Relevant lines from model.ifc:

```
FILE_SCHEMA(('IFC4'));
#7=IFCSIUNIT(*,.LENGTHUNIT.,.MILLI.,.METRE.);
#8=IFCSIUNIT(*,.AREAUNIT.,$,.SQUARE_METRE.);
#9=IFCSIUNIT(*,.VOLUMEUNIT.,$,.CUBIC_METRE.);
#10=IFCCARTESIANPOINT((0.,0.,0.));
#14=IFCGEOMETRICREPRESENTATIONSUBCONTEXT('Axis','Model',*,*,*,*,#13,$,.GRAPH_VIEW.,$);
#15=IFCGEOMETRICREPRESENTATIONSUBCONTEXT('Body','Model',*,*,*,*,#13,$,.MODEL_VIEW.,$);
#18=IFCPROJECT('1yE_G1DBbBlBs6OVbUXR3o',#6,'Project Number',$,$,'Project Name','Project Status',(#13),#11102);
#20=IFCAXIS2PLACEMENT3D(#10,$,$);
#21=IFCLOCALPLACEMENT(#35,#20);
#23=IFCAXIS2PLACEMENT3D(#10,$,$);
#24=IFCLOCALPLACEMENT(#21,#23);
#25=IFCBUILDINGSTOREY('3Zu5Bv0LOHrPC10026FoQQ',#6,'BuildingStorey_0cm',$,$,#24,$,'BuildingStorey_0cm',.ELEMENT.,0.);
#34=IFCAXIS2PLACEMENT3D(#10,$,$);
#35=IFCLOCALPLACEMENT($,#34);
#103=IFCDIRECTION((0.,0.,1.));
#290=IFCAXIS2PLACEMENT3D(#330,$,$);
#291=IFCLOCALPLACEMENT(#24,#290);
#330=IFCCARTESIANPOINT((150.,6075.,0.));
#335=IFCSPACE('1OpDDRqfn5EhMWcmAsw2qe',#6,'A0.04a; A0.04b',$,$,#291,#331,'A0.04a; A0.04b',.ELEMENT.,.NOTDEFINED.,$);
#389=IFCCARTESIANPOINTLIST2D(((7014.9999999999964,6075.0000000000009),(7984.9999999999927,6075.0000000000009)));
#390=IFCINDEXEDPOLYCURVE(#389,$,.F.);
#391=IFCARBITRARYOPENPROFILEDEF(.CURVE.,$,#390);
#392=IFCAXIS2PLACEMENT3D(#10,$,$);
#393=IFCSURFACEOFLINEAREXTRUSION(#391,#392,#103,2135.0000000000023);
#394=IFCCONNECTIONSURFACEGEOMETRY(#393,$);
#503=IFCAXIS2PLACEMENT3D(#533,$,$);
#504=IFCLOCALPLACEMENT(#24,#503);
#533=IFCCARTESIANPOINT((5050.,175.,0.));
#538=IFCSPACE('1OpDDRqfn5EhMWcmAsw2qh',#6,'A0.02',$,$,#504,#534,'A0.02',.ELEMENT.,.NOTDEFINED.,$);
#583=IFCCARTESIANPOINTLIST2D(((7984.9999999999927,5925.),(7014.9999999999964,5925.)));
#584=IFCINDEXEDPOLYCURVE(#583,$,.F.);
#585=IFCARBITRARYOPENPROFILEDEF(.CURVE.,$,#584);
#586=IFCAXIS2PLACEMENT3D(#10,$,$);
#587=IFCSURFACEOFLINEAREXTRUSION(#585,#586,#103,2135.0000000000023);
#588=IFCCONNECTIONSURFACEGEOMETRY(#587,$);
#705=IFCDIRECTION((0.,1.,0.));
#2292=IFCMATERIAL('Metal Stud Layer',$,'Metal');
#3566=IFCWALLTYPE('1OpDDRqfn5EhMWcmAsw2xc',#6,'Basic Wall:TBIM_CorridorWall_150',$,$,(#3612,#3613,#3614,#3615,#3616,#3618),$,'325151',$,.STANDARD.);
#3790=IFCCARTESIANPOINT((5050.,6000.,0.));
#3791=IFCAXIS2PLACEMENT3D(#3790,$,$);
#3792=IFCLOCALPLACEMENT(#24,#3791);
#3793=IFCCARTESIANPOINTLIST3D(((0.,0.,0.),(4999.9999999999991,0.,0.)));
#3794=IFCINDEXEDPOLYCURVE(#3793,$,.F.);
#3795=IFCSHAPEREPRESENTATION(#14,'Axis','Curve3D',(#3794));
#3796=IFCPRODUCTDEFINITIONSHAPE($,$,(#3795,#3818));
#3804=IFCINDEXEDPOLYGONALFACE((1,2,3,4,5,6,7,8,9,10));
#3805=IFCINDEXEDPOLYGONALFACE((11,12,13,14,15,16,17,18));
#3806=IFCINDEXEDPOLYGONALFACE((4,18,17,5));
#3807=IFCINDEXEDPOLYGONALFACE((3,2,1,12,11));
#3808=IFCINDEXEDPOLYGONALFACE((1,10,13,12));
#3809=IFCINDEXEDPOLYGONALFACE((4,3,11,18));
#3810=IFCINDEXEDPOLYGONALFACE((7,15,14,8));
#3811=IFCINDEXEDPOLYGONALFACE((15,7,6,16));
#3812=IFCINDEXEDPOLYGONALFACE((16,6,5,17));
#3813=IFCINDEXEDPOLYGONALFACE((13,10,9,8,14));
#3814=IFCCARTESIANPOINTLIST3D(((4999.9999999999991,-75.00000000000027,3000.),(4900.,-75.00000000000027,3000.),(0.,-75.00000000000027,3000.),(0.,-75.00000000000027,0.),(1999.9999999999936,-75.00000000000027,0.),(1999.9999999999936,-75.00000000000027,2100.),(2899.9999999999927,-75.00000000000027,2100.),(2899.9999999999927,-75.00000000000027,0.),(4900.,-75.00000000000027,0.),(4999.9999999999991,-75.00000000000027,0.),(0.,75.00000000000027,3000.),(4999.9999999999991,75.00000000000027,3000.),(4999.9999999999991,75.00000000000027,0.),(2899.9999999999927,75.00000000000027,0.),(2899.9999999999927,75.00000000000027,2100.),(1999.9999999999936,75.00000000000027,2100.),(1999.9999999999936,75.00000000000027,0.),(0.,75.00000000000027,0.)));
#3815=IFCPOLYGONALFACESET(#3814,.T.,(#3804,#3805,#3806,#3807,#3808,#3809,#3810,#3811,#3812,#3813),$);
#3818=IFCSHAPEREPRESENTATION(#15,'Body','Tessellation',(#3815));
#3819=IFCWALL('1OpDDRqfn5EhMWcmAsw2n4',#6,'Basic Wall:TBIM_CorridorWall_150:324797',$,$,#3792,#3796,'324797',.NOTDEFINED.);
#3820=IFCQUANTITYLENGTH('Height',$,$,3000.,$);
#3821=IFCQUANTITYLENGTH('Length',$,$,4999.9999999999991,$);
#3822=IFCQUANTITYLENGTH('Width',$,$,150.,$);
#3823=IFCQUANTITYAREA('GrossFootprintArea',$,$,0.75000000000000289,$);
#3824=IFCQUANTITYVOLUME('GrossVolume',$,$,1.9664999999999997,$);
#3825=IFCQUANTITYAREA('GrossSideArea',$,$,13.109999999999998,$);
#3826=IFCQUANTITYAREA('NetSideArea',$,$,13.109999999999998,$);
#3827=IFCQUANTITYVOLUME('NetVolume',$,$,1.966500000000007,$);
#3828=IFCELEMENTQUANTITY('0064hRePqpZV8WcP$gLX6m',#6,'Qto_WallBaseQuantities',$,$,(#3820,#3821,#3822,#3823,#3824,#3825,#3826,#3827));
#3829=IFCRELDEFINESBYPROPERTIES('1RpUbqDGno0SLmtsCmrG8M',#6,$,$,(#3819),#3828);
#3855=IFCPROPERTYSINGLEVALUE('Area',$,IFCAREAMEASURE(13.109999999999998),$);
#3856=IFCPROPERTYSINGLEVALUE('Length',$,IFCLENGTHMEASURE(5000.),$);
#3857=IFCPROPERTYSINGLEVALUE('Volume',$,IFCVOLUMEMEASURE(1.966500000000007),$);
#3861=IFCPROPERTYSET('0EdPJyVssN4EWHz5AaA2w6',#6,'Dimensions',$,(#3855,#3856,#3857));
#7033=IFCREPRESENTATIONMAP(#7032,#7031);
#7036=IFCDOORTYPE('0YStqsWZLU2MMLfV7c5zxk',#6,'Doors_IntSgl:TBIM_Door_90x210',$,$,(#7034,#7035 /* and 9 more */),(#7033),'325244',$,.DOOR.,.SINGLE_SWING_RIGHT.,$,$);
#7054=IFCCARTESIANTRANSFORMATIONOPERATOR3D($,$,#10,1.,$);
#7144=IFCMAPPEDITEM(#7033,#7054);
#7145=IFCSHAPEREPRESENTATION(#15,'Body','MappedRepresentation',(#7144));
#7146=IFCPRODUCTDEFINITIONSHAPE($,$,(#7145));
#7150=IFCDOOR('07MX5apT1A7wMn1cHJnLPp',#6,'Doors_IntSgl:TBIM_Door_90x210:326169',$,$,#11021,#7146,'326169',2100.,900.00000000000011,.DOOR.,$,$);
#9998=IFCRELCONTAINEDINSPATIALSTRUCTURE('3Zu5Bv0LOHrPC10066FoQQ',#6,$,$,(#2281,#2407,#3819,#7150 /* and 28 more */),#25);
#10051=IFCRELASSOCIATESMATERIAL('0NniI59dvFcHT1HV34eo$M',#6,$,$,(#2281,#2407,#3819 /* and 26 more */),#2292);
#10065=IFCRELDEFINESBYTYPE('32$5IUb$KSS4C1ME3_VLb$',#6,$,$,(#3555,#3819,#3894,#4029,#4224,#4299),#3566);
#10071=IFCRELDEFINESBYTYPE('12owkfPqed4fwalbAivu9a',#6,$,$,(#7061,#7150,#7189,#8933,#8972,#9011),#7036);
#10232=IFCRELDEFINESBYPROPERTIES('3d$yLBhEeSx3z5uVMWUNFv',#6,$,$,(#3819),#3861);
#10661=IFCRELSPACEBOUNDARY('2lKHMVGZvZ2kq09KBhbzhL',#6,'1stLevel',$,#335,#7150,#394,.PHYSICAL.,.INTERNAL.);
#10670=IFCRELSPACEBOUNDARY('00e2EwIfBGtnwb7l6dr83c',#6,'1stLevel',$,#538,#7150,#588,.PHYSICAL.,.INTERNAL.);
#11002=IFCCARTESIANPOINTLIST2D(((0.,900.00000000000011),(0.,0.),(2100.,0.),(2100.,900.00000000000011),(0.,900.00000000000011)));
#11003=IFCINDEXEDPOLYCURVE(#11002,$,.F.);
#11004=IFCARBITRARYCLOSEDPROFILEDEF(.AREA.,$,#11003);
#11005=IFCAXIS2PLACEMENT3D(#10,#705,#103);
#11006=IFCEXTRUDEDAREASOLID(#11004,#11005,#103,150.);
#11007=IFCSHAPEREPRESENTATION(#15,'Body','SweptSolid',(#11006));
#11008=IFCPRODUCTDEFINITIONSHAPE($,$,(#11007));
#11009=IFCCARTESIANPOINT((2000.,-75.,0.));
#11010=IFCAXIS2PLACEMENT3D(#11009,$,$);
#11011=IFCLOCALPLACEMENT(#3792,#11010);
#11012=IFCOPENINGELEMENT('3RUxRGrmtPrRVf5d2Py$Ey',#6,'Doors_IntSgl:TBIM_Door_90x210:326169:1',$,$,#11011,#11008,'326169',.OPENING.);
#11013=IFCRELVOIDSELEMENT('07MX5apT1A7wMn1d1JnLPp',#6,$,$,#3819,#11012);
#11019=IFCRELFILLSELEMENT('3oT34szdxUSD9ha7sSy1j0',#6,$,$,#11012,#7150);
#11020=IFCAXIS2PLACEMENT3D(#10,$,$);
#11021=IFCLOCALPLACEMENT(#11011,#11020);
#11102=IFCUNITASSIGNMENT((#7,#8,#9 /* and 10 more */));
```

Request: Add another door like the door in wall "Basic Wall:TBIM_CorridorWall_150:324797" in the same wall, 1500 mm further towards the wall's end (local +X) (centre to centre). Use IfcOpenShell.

```python
import numpy as np
import ifcopenshell
import ifcopenshell.api.feature
import ifcopenshell.api.geometry
import ifcopenshell.api.pset
import ifcopenshell.api.root
import ifcopenshell.geom
import ifcopenshell.util.element
import ifcopenshell.util.placement
import ifcopenshell.util.shape
import ifcopenshell.util.unit

model = ifcopenshell.open("model.ifc")
unit_scale = ifcopenshell.util.unit.calculate_unit_scale(model)
area_scale = ifcopenshell.util.unit.calculate_unit_scale(model, "AREAUNIT")
volume_scale = ifcopenshell.util.unit.calculate_unit_scale(model, "VOLUMEUNIT")
settings = ifcopenshell.geom.settings()


def volume(element):
    """Net volume in cubic metres, openings subtracted."""
    shape = ifcopenshell.geom.create_shape(settings, element)
    return ifcopenshell.util.shape.get_volume(shape.geometry)


def reuse_history(source, copy):
    """copy_class also copies each property set's owner history, people and application; keep the originals."""
    for rel in copy.IsDefinedBy:
        if rel.is_a("IfcRelDefinesByProperties") and (history := rel.RelatingPropertyDefinition.OwnerHistory):
            rel.RelatingPropertyDefinition.OwnerHistory = source.OwnerHistory
            ifcopenshell.util.element.remove_deep2(model, history)


door = model.by_guid("07MX5apT1A7wMn1cHJnLPp")
opening = door.FillsVoids[0].RelatingOpeningElement
wall = opening.VoidsElements[0].RelatingBuildingElement
before = volume(wall)
shift = ifcopenshell.util.placement.get_local_placement(wall.ObjectPlacement)[:3, 0] * 1.5 / unit_scale

# copy_class copies the void relationship, type, container and properties, but no geometry.
new_opening = ifcopenshell.api.root.copy_class(model, product=opening)
new_opening.Representation = ifcopenshell.util.element.copy_deep(
    model, opening.Representation, exclude=["IfcGeometricRepresentationContext", "IfcRepresentationMap"]
)
new_opening.Name = "Doors_IntSgl:TBIM_Door_90x210"
new_opening.Tag = None
reuse_history(opening, new_opening)
new_door = ifcopenshell.api.root.copy_class(model, product=door)
new_door.Representation = ifcopenshell.util.element.copy_deep(
    model, door.Representation, exclude=["IfcGeometricRepresentationContext", "IfcRepresentationMap"]
)
new_door.Name = "Doors_IntSgl:TBIM_Door_90x210"
new_door.Tag = None
reuse_history(door, new_door)
ifcopenshell.api.feature.add_filling(model, opening=new_opening, element=new_door)

for old, new in ((opening, new_opening), (door, new_door)):
    matrix = ifcopenshell.util.placement.get_local_placement(old.ObjectPlacement)
    matrix[:3, 3] += shift
    ifcopenshell.api.geometry.edit_object_placement(model, product=new, matrix=matrix, is_si=False)

# The copied space boundaries still share their surfaces with the original.
for rel in new_door.ProvidesBoundaries:
    if rel.ConnectionGeometry:
        rel.ConnectionGeometry = ifcopenshell.util.element.copy_deep(model, rel.ConnectionGeometry)

# Space boundary surfaces are stored in each space's coordinates; move them too.
for rel in new_door.ProvidesBoundaries:
    if not rel.ConnectionGeometry:
        continue
    surface = rel.ConnectionGeometry.SurfaceOnRelatingElement
    space_matrix = ifcopenshell.util.placement.get_local_placement(rel.RelatingSpace.ObjectPlacement)
    point = np.array(surface.Position.Location.Coordinates) + space_matrix[:3, :3].T @ shift
    surface.Position = model.createIfcAxis2Placement3D(
        model.createIfcCartesianPoint(point.tolist()), surface.Position.Axis, surface.Position.RefDirection
    )

after = volume(wall)
thickness = 0.15  # wall thickness in metres

# Update the wall's stored quantities.
qto = model.by_id(ifcopenshell.util.element.get_pset(wall, "Qto_WallBaseQuantities", should_inherit=False)["id"])
ifcopenshell.api.pset.edit_qto(model, qto=qto, properties={
    "NetSideArea": after / thickness / area_scale,
    "NetVolume": after / volume_scale,
})
pset = model.by_id(ifcopenshell.util.element.get_pset(wall, "Dimensions", should_inherit=False)["id"])
ifcopenshell.api.pset.edit_pset(model, pset=pset, properties={
    "Area": model.create_entity("IfcAreaMeasure", after / thickness / area_scale),
    "Volume": model.create_entity("IfcVolumeMeasure", after / volume_scale),
})

print(f"wall volume {before:.3f} -> {after:.3f} m3")

model.write("model_rev.ifc")
```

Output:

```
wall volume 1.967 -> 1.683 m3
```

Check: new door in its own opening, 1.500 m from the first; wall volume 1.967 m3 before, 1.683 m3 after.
